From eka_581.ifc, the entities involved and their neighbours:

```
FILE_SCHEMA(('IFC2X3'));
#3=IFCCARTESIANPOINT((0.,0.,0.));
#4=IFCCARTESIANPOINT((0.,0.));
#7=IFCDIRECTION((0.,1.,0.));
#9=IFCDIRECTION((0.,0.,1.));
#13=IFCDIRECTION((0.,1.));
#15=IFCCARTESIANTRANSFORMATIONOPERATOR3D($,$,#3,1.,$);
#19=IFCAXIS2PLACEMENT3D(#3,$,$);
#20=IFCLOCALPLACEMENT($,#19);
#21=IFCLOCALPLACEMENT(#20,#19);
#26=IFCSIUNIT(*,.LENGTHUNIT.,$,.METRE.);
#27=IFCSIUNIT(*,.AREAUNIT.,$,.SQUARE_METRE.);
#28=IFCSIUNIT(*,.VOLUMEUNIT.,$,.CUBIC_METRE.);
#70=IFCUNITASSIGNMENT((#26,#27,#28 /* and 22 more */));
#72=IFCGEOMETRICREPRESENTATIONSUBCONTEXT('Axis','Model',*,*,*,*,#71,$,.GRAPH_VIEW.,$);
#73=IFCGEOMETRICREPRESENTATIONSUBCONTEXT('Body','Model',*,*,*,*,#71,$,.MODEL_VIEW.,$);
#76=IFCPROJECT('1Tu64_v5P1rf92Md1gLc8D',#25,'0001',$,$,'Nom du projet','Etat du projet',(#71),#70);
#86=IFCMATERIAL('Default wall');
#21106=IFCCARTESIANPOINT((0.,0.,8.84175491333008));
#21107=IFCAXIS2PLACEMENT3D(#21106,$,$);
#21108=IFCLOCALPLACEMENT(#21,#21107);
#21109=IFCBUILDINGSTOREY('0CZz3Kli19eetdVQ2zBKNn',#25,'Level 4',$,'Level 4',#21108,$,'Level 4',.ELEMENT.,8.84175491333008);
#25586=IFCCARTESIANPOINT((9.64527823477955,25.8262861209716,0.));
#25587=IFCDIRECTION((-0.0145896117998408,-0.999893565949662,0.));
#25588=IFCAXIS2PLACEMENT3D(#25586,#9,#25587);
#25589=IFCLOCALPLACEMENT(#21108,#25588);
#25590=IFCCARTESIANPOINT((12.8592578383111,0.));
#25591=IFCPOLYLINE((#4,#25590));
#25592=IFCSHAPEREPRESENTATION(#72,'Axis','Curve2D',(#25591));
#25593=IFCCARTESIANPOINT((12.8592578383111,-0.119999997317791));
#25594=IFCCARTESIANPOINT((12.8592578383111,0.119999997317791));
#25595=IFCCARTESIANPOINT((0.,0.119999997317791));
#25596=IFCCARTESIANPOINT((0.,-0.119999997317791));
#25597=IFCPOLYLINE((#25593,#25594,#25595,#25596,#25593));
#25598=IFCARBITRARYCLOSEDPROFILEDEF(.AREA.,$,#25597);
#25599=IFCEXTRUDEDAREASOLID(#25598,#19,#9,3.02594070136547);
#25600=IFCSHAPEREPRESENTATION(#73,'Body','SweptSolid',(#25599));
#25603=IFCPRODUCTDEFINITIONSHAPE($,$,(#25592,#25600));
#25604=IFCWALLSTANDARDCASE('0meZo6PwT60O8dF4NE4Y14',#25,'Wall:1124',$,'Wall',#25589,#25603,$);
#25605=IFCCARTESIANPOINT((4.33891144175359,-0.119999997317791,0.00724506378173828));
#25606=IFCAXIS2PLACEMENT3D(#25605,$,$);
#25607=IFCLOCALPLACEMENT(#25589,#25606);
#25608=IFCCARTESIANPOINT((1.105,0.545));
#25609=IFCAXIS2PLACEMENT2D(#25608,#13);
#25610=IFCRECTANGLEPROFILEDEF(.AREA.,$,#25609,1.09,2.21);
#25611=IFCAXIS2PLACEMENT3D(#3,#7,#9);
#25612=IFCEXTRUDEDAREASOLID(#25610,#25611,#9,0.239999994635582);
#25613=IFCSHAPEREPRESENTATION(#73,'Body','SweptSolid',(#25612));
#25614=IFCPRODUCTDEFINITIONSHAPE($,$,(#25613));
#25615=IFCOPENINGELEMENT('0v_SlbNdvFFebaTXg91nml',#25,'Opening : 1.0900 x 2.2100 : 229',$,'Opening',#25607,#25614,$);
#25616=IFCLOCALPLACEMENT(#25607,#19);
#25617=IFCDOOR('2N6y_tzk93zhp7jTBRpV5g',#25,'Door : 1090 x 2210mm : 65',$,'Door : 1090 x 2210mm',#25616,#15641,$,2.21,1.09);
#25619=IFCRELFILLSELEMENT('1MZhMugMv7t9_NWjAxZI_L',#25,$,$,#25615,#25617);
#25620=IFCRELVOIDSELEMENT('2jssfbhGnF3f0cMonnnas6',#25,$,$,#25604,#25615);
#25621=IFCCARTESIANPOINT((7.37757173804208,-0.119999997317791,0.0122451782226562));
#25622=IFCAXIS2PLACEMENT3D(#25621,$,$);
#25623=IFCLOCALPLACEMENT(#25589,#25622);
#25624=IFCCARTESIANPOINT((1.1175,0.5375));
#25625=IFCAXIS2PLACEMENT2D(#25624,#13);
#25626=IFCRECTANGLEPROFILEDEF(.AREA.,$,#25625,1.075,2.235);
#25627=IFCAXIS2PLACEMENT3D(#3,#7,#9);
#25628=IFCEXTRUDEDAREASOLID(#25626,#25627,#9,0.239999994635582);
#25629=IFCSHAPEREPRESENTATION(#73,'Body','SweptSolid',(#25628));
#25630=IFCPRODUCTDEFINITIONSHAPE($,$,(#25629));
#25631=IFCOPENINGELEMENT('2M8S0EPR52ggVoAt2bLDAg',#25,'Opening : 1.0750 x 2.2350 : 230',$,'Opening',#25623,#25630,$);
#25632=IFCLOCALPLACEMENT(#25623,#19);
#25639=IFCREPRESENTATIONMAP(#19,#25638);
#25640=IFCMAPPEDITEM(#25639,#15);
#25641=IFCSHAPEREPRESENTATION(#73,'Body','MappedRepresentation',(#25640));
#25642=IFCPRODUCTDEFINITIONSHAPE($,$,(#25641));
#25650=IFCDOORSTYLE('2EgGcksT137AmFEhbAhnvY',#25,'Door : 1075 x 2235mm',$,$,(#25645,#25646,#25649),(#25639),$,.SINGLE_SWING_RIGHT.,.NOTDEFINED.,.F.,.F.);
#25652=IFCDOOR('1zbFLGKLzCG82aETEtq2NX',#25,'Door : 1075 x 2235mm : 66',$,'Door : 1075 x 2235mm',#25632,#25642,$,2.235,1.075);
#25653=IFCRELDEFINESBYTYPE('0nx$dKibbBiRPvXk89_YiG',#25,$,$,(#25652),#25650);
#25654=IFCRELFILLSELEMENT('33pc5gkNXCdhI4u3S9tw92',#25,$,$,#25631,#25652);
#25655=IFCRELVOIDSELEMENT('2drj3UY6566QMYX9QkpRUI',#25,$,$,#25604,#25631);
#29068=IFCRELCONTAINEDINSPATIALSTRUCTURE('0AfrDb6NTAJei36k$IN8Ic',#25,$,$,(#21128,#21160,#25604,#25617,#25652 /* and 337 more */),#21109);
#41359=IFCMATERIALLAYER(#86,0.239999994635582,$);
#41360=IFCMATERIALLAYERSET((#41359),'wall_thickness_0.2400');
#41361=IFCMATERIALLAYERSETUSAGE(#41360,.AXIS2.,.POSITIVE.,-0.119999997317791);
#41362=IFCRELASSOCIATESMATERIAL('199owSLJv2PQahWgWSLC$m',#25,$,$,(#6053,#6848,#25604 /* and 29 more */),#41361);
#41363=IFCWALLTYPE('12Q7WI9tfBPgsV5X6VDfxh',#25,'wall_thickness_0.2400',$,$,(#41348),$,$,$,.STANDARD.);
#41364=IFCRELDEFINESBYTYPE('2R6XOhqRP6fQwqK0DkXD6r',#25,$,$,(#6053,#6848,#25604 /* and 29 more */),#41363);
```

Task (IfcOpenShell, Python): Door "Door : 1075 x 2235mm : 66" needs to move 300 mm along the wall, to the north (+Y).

```python
import ifcopenshell
import ifcopenshell.api.geometry
import ifcopenshell.util.placement

model = ifcopenshell.open("eka_581.ifc")

door = model.by_guid("1zbFLGKLzCG82aETEtq2NX")
opening = door.FillsVoids[0].RelatingOpeningElement
wall = opening.VoidsElements[0].RelatingBuildingElement

wall_matrix = ifcopenshell.util.placement.get_local_placement(wall.ObjectPlacement)
shift = wall_matrix[:3, 0] * -0.3
before = ifcopenshell.util.placement.get_local_placement(door.ObjectPlacement)[:3, 3].copy()

# The door is placed relative to its opening, so it follows when the opening moves.
matrix = ifcopenshell.util.placement.get_local_placement(opening.ObjectPlacement)
matrix[:3, 3] += shift
ifcopenshell.api.geometry.edit_object_placement(
    model, product=opening, matrix=matrix, is_si=False, should_transform_children=True
)

after = ifcopenshell.util.placement.get_local_placement(door.ObjectPlacement)[:3, 3]
print("door moved by", (after - before).round(3) + 0.0)

model.write("eka_581_rev.ifc")
```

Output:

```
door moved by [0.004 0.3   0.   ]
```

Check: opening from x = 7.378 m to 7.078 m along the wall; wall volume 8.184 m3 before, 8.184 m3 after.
